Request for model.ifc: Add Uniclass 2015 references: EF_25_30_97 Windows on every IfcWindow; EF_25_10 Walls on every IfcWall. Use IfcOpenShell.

First a look at what the model holds.

```python
import ifcopenshell

model = ifcopenshell.open("model.ifc")
print(model.schema)
print("classifications:", [c.Name for c in model.by_type("IfcClassification")])
for ifc_class in ("IfcDoor", "IfcRoof", "IfcStair", "IfcWall", "IfcWindow"):
    print(ifc_class, len(model.by_type(ifc_class)))
```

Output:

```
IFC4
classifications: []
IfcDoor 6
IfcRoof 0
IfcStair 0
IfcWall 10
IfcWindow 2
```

```python
import ifcopenshell
import ifcopenshell.api.classification

model = ifcopenshell.open("model.ifc")

system = ifcopenshell.api.classification.add_classification(model, classification="Uniclass 2015")

codes = {
    "IfcWindow": ("EF_25_30_97", "Windows"),
    "IfcWall": ("EF_25_10", "Walls"),
}
for ifc_class, (code, name) in codes.items():
    products = model.by_type(ifc_class)
    ifcopenshell.api.classification.add_reference(
        model, products=products, classification=system, identification=code, name=name
    )
    print(code, len(products))

model.write("model_edited.ifc")
```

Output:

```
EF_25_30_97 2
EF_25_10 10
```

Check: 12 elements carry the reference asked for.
